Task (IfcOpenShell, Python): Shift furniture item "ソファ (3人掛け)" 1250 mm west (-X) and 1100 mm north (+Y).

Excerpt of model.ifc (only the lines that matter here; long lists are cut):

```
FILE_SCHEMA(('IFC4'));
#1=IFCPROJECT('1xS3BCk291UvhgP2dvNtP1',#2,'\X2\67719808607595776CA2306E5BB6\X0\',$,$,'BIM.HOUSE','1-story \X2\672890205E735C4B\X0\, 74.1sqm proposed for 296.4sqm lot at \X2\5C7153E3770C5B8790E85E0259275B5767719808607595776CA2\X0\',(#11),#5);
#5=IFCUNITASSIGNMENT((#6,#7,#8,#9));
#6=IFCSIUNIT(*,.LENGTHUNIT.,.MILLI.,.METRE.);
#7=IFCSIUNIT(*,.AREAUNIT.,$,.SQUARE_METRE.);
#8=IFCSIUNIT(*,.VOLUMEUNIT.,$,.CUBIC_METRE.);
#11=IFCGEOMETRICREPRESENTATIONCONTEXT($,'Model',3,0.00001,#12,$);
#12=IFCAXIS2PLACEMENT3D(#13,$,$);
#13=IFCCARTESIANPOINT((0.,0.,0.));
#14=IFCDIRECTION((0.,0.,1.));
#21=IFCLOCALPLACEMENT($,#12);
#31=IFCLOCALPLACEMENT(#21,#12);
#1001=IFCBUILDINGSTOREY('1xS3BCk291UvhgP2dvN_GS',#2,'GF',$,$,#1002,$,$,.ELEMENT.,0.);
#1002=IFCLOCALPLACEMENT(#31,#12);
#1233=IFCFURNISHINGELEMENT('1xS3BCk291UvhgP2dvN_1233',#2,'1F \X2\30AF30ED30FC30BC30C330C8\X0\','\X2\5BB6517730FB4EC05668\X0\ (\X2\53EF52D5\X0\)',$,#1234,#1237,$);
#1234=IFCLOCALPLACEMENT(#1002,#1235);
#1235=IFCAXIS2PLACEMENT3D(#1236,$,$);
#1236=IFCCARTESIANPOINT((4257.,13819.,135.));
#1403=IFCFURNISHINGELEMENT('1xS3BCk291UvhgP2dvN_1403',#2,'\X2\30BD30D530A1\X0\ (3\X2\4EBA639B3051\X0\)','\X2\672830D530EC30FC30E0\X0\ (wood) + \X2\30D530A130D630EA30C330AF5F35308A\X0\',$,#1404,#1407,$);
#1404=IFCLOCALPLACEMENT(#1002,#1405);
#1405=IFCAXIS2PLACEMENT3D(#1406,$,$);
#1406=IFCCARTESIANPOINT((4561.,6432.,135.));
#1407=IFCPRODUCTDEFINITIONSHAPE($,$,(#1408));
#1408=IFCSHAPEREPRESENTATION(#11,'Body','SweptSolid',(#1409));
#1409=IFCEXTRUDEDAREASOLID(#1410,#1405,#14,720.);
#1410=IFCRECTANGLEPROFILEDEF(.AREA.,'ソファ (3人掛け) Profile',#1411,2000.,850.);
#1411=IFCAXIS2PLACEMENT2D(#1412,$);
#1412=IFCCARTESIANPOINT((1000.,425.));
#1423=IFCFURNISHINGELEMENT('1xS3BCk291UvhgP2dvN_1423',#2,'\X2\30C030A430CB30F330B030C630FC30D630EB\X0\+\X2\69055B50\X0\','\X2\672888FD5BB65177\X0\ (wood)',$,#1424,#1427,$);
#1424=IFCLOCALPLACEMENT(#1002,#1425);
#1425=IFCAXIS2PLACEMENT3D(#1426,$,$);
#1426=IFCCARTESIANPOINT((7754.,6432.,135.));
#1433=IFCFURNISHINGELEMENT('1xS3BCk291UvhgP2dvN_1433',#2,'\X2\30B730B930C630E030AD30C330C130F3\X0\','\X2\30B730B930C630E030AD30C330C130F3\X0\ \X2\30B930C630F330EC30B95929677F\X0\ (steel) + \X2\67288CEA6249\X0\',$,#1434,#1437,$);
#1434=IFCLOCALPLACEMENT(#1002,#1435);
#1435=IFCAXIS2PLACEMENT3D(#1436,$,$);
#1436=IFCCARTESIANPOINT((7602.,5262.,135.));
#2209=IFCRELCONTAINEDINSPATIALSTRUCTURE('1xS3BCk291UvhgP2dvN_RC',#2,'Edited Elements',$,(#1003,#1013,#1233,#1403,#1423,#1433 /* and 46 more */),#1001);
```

```python
import ifcopenshell
import ifcopenshell.api.geometry
import ifcopenshell.util.placement
import ifcopenshell.util.unit

model = ifcopenshell.open("model.ifc")
unit_scale = ifcopenshell.util.unit.calculate_unit_scale(model)

item = model.by_id(1403)
matrix = ifcopenshell.util.placement.get_local_placement(item.ObjectPlacement)
matrix[0, 3] -= 1.25 / unit_scale
matrix[1, 3] += 1.1 / unit_scale
ifcopenshell.api.geometry.edit_object_placement(model, product=item, matrix=matrix, is_si=False)

print(ifcopenshell.util.placement.get_local_placement(item.ObjectPlacement).round(3) + 0.0)

model.write("model_edited.ifc")
```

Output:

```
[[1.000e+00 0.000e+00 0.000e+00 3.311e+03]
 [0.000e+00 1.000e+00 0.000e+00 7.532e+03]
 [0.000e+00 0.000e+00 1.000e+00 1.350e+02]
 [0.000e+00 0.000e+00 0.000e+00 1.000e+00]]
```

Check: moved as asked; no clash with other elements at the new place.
